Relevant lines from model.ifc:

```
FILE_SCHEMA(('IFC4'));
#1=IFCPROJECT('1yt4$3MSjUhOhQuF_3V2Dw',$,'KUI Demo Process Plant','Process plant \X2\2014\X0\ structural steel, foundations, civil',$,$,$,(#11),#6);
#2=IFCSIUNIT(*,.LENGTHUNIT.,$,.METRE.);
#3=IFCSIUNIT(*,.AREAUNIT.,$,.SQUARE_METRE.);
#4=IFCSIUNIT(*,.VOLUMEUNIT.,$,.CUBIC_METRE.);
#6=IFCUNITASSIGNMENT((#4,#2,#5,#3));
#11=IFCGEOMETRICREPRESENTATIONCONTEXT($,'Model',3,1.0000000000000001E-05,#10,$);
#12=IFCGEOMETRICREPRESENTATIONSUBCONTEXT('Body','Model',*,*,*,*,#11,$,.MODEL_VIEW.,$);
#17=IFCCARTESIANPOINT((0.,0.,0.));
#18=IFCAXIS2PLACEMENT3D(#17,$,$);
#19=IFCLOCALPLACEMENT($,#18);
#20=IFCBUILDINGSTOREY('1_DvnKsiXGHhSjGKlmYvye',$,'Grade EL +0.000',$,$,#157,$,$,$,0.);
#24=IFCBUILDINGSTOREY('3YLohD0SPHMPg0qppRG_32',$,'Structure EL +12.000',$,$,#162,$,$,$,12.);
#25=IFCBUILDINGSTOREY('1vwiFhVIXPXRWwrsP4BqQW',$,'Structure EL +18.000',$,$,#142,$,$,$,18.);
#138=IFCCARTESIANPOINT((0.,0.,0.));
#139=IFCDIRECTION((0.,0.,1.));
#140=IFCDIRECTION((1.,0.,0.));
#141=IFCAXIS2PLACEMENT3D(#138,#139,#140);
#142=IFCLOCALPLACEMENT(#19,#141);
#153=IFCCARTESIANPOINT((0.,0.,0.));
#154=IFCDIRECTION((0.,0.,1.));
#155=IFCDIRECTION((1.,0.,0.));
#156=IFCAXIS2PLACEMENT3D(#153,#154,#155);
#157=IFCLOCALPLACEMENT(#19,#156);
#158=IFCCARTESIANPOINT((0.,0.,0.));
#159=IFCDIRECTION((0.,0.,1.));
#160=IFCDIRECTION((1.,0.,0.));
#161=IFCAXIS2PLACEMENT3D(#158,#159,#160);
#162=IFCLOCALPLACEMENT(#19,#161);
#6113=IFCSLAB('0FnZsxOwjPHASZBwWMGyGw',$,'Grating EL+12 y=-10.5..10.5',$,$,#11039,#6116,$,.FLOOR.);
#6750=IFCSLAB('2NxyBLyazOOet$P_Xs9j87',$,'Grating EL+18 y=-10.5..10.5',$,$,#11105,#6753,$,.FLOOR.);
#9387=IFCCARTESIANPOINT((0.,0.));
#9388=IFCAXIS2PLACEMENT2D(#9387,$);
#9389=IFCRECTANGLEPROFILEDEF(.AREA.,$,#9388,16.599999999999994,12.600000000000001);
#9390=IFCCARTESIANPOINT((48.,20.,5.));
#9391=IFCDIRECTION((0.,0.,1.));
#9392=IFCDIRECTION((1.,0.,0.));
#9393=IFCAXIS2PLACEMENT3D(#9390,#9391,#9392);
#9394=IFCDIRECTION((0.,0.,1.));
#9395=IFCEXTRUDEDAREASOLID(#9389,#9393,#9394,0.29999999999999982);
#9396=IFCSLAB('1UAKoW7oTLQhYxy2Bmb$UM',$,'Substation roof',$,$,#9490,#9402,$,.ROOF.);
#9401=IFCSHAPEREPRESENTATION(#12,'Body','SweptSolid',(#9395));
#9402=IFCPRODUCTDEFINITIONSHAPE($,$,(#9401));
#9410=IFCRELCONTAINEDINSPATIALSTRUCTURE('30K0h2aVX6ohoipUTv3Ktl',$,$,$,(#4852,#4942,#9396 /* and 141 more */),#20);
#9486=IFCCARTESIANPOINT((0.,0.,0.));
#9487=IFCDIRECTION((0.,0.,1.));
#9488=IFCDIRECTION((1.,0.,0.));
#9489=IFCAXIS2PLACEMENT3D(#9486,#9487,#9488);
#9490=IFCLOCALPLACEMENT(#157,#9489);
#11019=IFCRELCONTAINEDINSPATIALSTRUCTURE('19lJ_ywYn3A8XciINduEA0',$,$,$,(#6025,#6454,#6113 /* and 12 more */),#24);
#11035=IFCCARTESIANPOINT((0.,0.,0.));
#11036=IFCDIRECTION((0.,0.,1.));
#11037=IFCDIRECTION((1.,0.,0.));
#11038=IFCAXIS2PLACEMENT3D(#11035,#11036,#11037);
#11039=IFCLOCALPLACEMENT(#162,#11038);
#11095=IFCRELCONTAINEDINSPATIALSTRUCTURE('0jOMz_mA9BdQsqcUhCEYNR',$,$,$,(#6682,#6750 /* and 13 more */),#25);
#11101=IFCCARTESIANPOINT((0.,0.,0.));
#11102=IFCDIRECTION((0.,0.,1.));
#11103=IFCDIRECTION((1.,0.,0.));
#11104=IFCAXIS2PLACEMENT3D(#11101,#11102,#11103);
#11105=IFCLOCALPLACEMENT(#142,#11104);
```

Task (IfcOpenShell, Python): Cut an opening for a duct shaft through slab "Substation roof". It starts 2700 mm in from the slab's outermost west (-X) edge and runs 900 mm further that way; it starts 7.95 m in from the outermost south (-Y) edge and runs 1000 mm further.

```python
import numpy as np
import ifcopenshell
import ifcopenshell.api.feature
import ifcopenshell.api.geometry
import ifcopenshell.api.root
import ifcopenshell.geom
import ifcopenshell.util.placement
import ifcopenshell.util.representation
import ifcopenshell.util.shape
import ifcopenshell.util.unit

model = ifcopenshell.open("model.ifc")
unit_scale = ifcopenshell.util.unit.calculate_unit_scale(model)
settings = ifcopenshell.geom.settings()


def volume(element):
    """Net volume in cubic metres, openings subtracted."""
    shape = ifcopenshell.geom.create_shape(settings, element)
    return ifcopenshell.util.shape.get_volume(shape.geometry)


slab = model.by_id(9396)
before = volume(slab)

# Extent in the slab's own axes, in metres. The edges named are its -X and -Y sides.
slab_shape = ifcopenshell.geom.create_shape(settings, slab)
vertices = ifcopenshell.util.shape.get_vertices(slab_shape.geometry)
x_min, y_min, bottom = vertices.min(axis=0)
top = vertices[:, 2].max()

opening = ifcopenshell.api.root.create_entity(model, ifc_class="IfcOpeningElement", name="Duct shaft opening", predefined_type="OPENING")
context = ifcopenshell.util.representation.get_context(model, "Model", "Body", "MODEL_VIEW")
width, depth = 0.9, 1
outline = [(0.0, 0.0), (width, 0.0), (width, depth), (0.0, depth), (0.0, 0.0)]
# Overshoot both faces by 50 mm so the cut is clean.
shape = ifcopenshell.api.geometry.add_slab_representation(
    model, context=context, depth=top - bottom + 0.1, polyline=outline
)
ifcopenshell.api.geometry.assign_representation(model, product=opening, representation=shape)

matrix = ifcopenshell.util.placement.get_local_placement(slab.ObjectPlacement)
matrix[:, 3] = matrix @ np.append(np.array([x_min + 2.7, y_min + 7.95, bottom - 0.05]) / unit_scale, 1.0)
ifcopenshell.api.geometry.edit_object_placement(model, product=opening, matrix=matrix, is_si=False)
ifcopenshell.api.feature.add_feature(model, feature=opening, element=slab)

after = volume(slab)

print(f"slab volume {before:.3f} -> {after:.3f} m3")

model.write("model_rev.ifc")
```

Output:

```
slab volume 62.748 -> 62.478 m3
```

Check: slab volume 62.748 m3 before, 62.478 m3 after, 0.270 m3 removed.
